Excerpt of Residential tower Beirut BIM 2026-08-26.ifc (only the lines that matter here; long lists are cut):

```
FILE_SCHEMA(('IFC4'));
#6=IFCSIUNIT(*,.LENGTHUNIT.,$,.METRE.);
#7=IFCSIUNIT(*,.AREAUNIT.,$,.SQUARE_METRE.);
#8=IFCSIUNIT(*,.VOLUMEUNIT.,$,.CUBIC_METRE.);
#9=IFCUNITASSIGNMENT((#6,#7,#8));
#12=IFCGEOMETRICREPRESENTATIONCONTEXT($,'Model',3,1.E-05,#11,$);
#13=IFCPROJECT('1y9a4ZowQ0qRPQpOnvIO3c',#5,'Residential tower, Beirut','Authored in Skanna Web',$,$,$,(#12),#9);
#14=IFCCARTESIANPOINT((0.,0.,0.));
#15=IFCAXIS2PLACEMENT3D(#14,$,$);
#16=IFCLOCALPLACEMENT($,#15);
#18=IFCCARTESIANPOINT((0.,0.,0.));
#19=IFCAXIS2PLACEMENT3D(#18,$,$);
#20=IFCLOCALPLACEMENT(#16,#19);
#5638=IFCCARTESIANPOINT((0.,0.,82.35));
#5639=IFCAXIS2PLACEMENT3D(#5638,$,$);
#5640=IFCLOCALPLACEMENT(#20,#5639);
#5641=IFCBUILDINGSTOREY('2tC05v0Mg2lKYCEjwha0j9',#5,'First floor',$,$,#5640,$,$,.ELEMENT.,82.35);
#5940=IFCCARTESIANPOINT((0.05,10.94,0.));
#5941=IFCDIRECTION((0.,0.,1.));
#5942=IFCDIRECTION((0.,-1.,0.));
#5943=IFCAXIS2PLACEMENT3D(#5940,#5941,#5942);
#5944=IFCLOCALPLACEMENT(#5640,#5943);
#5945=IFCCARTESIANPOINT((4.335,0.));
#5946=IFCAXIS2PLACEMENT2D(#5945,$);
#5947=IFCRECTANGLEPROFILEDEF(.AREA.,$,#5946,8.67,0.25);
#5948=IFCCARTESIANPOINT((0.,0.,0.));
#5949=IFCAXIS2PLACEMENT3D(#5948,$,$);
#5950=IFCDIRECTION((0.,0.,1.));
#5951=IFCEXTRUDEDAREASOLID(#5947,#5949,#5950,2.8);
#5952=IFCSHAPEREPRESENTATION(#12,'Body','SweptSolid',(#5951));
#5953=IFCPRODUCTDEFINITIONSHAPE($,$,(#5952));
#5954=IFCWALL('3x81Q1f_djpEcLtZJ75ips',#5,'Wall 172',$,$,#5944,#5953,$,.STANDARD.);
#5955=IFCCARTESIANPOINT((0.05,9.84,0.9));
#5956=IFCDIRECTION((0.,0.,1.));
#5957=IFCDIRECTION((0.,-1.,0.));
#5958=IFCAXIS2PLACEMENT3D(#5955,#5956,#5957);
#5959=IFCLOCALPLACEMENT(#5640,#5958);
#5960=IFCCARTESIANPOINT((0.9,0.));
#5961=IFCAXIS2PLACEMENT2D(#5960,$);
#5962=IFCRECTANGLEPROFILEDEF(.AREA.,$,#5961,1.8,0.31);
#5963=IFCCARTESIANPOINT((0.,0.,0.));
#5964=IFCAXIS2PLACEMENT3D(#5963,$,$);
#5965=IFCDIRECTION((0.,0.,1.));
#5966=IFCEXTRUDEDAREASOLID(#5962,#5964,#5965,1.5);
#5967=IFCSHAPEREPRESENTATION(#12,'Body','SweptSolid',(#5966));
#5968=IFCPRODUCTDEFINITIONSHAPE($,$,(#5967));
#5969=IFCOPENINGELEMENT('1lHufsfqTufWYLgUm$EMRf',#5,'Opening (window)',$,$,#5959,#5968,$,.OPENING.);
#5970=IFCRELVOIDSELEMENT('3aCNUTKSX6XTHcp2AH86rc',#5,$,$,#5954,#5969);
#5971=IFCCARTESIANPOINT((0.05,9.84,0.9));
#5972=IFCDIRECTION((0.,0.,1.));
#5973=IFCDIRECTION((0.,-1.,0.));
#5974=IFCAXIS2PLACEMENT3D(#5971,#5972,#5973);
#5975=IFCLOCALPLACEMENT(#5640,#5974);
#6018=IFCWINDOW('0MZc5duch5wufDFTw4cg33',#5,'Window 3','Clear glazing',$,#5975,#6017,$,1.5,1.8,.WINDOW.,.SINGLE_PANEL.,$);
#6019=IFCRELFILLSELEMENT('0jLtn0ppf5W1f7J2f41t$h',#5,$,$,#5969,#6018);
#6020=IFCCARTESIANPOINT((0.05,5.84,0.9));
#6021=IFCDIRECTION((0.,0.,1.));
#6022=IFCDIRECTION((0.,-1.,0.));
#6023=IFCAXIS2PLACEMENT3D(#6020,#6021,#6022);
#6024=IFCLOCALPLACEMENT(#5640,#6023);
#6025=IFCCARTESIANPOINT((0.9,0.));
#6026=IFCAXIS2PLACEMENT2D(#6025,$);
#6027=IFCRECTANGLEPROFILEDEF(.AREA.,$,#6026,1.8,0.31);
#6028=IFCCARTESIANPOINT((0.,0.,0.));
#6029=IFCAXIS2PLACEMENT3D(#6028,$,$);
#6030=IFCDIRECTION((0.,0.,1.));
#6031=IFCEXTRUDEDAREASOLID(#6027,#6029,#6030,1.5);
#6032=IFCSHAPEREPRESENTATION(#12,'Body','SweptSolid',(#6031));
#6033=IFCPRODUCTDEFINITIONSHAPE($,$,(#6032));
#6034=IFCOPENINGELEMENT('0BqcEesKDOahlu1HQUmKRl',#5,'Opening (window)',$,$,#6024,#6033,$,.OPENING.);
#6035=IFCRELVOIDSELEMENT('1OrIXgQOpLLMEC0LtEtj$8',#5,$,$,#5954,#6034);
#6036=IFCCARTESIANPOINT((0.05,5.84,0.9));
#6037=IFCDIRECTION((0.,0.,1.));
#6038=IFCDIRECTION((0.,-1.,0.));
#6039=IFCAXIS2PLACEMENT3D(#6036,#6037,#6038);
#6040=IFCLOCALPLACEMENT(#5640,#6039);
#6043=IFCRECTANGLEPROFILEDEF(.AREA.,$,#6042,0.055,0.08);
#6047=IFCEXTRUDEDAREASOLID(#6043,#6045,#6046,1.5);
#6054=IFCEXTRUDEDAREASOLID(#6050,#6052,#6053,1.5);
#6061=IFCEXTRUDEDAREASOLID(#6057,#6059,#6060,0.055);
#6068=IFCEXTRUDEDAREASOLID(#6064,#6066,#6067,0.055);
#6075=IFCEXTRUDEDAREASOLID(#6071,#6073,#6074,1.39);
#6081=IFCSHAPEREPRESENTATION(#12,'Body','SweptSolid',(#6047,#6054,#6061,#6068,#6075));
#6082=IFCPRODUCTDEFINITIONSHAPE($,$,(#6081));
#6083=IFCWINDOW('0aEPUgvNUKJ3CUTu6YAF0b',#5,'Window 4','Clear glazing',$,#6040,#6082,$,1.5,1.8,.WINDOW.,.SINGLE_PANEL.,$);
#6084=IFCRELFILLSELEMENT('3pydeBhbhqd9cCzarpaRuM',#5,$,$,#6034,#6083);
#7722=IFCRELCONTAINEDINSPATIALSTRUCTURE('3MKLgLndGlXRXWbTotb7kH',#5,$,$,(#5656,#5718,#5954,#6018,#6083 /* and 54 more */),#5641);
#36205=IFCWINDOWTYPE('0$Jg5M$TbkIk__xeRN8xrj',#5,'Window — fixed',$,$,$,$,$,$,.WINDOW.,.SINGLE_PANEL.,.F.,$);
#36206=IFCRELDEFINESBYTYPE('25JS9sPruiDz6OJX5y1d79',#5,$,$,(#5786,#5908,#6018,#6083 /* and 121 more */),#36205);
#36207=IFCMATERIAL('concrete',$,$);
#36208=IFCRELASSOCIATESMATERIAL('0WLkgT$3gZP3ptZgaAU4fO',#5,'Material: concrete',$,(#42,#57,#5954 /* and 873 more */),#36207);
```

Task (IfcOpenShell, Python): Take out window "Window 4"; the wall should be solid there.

```python
import ifcopenshell
import ifcopenshell.api.feature
import ifcopenshell.api.root
import ifcopenshell.geom
import ifcopenshell.util.shape

model = ifcopenshell.open("Residential tower Beirut BIM 2026-08-26.ifc")
settings = ifcopenshell.geom.settings()


def volume(element):
    """Net volume in cubic metres, openings subtracted."""
    shape = ifcopenshell.geom.create_shape(settings, element)
    return ifcopenshell.util.shape.get_volume(shape.geometry)


window = model.by_guid("0aEPUgvNUKJ3CUTu6YAF0b")
opening = window.FillsVoids[0].RelatingOpeningElement
wall = opening.VoidsElements[0].RelatingBuildingElement
before = volume(wall)

ifcopenshell.api.root.remove_product(model, product=window)
ifcopenshell.api.feature.remove_feature(model, feature=opening)

after = volume(wall)

print(f"wall volume {before:.3f} -> {after:.3f} m3")

model.write("Residential tower Beirut BIM 2026-08-26_updated.ifc")
```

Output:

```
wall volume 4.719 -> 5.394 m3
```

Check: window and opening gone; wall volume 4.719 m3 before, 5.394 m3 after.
